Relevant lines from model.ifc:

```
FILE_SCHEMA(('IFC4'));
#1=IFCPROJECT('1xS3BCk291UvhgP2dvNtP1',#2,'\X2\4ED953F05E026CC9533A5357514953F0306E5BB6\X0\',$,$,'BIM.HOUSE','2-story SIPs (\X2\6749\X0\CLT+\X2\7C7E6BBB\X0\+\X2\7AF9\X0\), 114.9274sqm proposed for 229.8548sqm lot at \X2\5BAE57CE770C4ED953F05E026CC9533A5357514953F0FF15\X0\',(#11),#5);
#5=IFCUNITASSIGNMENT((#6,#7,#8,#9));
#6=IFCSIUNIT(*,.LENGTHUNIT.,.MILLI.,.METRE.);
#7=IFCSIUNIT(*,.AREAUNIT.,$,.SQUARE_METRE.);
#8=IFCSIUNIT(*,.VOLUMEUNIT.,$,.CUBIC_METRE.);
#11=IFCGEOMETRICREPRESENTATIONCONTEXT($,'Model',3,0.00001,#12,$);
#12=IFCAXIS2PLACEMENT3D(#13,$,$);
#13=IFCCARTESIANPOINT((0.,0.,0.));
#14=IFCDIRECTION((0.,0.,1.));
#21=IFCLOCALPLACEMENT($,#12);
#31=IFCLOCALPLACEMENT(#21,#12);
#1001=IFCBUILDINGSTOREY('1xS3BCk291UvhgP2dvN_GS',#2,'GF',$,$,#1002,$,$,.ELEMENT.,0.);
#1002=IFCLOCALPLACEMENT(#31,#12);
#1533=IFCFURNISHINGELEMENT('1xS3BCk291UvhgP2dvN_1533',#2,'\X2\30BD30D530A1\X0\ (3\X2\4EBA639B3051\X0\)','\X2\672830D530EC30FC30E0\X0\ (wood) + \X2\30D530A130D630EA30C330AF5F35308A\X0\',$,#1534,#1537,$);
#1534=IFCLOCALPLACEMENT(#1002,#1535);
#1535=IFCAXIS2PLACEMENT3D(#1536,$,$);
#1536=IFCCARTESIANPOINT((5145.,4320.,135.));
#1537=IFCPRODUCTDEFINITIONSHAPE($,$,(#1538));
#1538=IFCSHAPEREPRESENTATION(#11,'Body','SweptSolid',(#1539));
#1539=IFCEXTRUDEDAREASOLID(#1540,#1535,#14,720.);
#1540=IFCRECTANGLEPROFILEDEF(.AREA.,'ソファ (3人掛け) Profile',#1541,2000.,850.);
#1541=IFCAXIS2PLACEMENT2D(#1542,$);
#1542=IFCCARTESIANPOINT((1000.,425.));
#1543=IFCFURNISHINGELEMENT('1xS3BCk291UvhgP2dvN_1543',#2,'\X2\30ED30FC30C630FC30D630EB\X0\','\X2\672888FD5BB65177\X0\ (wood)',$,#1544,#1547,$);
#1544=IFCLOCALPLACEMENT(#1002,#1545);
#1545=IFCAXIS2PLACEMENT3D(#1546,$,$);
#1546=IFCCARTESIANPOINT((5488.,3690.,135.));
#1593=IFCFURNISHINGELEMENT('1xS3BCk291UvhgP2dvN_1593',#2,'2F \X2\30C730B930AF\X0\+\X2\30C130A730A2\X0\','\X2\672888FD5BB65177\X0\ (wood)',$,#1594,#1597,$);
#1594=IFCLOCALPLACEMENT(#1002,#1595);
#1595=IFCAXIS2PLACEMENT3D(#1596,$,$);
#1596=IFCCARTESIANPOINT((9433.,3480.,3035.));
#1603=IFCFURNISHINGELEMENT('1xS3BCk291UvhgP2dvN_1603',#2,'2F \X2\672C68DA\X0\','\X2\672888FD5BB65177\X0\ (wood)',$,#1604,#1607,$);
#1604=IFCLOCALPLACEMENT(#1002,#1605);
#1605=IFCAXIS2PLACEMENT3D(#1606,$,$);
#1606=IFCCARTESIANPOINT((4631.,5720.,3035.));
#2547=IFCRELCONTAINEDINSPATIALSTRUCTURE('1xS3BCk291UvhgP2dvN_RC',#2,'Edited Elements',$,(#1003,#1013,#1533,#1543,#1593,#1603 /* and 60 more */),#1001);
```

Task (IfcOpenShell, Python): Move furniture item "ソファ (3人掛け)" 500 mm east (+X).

```python
import ifcopenshell
import ifcopenshell.api.geometry
import ifcopenshell.util.placement
import ifcopenshell.util.unit

model = ifcopenshell.open("model.ifc")
unit_scale = ifcopenshell.util.unit.calculate_unit_scale(model)

item = model.by_guid("1xS3BCk291UvhgP2dvN_1533")
matrix = ifcopenshell.util.placement.get_local_placement(item.ObjectPlacement)
matrix[0, 3] += 0.5 / unit_scale
ifcopenshell.api.geometry.edit_object_placement(model, product=item, matrix=matrix, is_si=False)

print(ifcopenshell.util.placement.get_local_placement(item.ObjectPlacement).round(3) + 0.0)

model.write("model-out.ifc")
```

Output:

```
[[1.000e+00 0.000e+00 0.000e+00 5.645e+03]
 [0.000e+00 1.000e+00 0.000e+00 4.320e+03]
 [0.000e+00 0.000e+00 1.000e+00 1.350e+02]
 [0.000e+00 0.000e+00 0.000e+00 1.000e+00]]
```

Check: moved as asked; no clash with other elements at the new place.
